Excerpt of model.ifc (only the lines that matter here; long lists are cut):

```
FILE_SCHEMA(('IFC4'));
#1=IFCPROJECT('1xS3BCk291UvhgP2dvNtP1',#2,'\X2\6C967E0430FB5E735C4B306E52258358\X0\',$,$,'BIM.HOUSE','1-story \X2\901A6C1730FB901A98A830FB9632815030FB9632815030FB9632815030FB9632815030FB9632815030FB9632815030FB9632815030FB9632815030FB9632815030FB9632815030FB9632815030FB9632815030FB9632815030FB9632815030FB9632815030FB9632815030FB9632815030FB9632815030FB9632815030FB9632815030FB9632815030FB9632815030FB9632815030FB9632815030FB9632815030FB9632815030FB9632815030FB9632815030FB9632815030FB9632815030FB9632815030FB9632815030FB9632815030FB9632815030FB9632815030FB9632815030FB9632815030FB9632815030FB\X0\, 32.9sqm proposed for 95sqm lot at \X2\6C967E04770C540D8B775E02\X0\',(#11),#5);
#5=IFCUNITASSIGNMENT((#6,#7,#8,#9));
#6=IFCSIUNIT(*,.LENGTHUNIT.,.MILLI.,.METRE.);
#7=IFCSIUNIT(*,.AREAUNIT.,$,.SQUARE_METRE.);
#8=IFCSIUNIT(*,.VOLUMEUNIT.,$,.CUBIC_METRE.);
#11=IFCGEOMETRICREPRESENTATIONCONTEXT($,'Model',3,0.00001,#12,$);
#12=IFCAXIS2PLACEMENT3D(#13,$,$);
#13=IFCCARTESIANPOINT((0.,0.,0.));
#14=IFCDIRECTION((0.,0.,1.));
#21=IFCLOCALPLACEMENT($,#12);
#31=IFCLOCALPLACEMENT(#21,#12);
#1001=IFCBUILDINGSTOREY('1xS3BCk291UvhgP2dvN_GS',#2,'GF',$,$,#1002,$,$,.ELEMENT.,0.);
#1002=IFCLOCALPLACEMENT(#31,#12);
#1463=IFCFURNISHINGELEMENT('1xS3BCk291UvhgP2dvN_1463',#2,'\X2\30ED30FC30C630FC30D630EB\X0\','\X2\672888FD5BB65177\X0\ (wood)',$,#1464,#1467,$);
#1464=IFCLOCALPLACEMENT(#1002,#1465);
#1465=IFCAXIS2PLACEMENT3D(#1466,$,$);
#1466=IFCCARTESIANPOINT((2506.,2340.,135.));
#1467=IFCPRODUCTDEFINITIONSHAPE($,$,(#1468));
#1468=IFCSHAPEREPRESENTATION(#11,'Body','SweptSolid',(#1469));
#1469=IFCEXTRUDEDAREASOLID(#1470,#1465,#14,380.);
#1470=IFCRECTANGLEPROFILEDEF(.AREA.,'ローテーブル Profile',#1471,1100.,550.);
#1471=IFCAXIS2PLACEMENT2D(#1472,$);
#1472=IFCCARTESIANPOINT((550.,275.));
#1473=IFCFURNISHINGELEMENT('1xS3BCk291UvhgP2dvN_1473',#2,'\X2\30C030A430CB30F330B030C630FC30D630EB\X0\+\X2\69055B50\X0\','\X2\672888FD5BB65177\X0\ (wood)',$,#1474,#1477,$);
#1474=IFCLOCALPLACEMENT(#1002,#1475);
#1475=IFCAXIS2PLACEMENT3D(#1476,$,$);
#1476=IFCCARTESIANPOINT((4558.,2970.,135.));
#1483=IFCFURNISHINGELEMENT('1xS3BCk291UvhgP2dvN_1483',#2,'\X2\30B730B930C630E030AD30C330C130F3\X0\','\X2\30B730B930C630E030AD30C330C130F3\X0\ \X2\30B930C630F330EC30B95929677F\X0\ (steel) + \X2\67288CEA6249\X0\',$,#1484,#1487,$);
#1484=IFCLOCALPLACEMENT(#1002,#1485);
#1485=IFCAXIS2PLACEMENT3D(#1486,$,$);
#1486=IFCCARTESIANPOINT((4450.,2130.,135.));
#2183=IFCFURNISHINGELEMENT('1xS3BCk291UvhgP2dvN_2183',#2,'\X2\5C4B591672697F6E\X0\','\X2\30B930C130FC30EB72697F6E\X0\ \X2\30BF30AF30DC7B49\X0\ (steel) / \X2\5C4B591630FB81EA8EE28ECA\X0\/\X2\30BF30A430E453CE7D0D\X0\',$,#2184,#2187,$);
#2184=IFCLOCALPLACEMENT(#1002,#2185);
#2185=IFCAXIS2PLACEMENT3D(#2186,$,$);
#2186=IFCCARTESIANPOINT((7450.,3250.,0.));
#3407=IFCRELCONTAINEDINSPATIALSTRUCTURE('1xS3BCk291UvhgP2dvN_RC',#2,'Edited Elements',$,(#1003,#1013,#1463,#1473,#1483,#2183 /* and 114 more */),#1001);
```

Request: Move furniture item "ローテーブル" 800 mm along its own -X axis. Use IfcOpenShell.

```python
import ifcopenshell
import ifcopenshell.api.geometry
import ifcopenshell.util.placement

model = ifcopenshell.open("model.ifc")

item = model.by_guid("1xS3BCk291UvhgP2dvN_1463")
matrix = ifcopenshell.util.placement.get_local_placement(item.ObjectPlacement)
matrix[:3, 3] -= matrix[:3, 0] * 800.0
ifcopenshell.api.geometry.edit_object_placement(model, product=item, matrix=matrix, is_si=False)

print(ifcopenshell.util.placement.get_local_placement(item.ObjectPlacement).round(3) + 0.0)

model.write("model_rev.ifc")
```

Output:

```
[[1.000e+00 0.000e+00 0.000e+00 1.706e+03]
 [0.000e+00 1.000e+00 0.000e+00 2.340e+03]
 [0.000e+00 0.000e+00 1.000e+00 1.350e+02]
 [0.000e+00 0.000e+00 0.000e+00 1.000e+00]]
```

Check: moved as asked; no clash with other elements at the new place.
